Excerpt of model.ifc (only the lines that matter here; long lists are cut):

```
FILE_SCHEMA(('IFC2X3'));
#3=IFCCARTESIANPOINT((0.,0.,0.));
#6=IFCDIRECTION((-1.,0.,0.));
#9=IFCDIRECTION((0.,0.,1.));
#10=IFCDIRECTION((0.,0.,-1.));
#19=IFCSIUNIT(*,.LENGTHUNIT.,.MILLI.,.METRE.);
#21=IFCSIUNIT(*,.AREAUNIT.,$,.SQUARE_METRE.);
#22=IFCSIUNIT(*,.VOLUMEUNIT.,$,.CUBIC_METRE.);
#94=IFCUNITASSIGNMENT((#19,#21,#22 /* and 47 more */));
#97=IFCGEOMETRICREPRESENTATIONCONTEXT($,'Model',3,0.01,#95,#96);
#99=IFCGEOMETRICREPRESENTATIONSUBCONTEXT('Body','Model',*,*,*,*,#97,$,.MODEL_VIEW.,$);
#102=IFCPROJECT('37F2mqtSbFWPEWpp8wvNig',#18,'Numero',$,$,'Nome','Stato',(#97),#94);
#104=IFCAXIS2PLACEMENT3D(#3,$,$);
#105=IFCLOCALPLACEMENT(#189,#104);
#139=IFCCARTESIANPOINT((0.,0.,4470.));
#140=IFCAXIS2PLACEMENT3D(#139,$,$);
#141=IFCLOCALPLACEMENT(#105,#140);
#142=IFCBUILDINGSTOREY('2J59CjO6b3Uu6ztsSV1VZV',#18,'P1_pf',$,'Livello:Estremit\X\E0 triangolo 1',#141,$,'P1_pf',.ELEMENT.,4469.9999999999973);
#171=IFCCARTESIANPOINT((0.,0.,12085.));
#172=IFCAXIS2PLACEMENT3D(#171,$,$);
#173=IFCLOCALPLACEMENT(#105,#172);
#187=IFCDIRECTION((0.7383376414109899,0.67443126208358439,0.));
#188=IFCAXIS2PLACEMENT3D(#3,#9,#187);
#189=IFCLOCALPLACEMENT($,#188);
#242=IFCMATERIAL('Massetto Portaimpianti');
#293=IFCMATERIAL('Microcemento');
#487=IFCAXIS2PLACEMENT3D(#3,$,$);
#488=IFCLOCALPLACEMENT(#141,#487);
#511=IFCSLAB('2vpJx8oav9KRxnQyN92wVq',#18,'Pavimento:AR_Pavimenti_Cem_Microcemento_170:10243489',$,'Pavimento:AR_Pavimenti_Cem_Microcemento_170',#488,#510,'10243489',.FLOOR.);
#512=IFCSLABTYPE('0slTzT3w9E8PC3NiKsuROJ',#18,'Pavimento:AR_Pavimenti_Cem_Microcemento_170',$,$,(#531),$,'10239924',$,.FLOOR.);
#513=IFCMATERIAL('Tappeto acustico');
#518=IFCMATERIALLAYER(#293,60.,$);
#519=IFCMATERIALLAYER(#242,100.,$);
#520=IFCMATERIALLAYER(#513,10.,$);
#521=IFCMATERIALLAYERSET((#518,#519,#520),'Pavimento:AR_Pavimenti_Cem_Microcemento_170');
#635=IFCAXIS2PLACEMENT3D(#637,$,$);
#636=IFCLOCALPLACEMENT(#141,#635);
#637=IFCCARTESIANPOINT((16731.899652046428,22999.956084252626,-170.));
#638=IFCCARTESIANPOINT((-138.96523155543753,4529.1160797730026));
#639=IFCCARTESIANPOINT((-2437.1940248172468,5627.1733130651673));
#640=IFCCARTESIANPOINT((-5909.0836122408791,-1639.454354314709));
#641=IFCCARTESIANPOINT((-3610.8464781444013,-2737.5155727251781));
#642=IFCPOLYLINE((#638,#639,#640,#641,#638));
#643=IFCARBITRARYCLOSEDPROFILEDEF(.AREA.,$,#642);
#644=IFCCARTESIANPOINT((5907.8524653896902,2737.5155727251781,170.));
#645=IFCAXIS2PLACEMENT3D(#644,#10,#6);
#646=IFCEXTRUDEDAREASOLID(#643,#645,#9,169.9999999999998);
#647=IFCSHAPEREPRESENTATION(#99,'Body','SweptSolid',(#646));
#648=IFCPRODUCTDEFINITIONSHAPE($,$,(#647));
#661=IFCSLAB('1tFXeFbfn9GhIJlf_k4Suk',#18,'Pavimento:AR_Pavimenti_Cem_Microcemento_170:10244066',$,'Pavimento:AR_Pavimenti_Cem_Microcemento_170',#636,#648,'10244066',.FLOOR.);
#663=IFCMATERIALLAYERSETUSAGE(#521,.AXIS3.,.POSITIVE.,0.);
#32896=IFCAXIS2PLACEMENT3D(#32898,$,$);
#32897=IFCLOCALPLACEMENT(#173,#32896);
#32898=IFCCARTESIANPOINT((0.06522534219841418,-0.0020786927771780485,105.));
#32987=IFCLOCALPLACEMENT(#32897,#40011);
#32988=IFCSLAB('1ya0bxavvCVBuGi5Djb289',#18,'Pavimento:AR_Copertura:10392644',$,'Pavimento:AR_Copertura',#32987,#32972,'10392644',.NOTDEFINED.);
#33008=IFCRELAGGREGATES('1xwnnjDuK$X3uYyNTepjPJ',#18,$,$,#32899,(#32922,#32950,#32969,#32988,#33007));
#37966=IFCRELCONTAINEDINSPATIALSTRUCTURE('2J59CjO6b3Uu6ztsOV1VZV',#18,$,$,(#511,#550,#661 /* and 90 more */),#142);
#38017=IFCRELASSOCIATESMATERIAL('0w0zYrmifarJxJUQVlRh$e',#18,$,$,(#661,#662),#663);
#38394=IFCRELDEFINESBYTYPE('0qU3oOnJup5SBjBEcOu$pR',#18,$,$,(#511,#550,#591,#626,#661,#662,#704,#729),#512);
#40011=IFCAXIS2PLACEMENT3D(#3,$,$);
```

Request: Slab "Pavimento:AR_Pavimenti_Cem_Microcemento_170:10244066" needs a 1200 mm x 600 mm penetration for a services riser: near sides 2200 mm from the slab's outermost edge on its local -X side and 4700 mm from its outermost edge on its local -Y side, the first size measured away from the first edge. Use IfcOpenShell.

```python
import numpy as np
import ifcopenshell
import ifcopenshell.api.feature
import ifcopenshell.api.geometry
import ifcopenshell.api.root
import ifcopenshell.geom
import ifcopenshell.util.placement
import ifcopenshell.util.representation
import ifcopenshell.util.shape
import ifcopenshell.util.unit

model = ifcopenshell.open("model.ifc")
unit_scale = ifcopenshell.util.unit.calculate_unit_scale(model)
settings = ifcopenshell.geom.settings()


def volume(element):
    """Net volume in cubic metres, openings subtracted."""
    shape = ifcopenshell.geom.create_shape(settings, element)
    return ifcopenshell.util.shape.get_volume(shape.geometry)


slab = model.by_guid("1tFXeFbfn9GhIJlf_k4Suk")
before = volume(slab)

# Extent in the slab's own axes, in metres. The edges named are its -X and -Y sides.
slab_shape = ifcopenshell.geom.create_shape(settings, slab)
vertices = ifcopenshell.util.shape.get_vertices(slab_shape.geometry)
x_min, y_min, bottom = vertices.min(axis=0)
top = vertices[:, 2].max()

opening = ifcopenshell.api.root.create_entity(model, ifc_class="IfcOpeningElement", name="Services riser opening")
context = ifcopenshell.util.representation.get_context(model, "Model", "Body", "MODEL_VIEW")
width, depth = 1.2, 0.6
outline = [(0.0, 0.0), (width, 0.0), (width, depth), (0.0, depth), (0.0, 0.0)]
# Overshoot both faces by 50 mm so the cut is clean.
shape = ifcopenshell.api.geometry.add_slab_representation(
    model, context=context, depth=top - bottom + 0.1, polyline=outline
)
ifcopenshell.api.geometry.assign_representation(model, product=opening, representation=shape)

matrix = ifcopenshell.util.placement.get_local_placement(slab.ObjectPlacement)
matrix[:, 3] = matrix @ np.append(np.array([x_min + 2.2, y_min + 4.7, bottom - 0.05]) / unit_scale, 1.0)
ifcopenshell.api.geometry.edit_object_placement(model, product=opening, matrix=matrix, is_si=False)
ifcopenshell.api.feature.add_feature(model, feature=opening, element=slab)

after = volume(slab)

print(f"slab volume {before:.3f} -> {after:.3f} m3")

model.write("model-out.ifc")
```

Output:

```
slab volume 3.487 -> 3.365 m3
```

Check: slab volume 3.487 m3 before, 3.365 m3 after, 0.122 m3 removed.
